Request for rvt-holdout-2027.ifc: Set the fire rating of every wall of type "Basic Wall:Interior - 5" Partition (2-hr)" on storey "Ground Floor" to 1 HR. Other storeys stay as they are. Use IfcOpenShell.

First a look at what the model holds.

```python
import ifcopenshell
import ifcopenshell.util.element

model = ifcopenshell.open("rvt-holdout-2027.ifc")
print(model.schema)
storey = next(s for s in model.by_type("IfcBuildingStorey") if s.Name == "Ground Floor")
walls = [e for e in ifcopenshell.util.element.get_decomposition(storey) if e.is_a("IfcWall")]
seen = {}
for e in walls:
    element_type = ifcopenshell.util.element.get_type(e)
    key = (element_type.Name if element_type != e and element_type else None, ifcopenshell.util.element.get_pset(e, "Pset_WallCommon", "FireRating"))
    seen[key] = seen.get(key, 0) + 1
for (name, value), count in sorted(seen.items(), key=str):
    print(count, "x", name, "|", value)
```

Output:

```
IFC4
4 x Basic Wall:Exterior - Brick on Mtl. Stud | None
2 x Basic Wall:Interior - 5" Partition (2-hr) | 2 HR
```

```python
import ifcopenshell
import ifcopenshell.api.pset
import ifcopenshell.util.element

model = ifcopenshell.open("rvt-holdout-2027.ifc")

storey = next(s for s in model.by_type("IfcBuildingStorey") if s.Name == "Ground Floor")
walls = [e for e in ifcopenshell.util.element.get_decomposition(storey) if e.is_a("IfcWall")]

count = 0
for e in walls:
    element_type = ifcopenshell.util.element.get_type(e)
    if element_type in (None, e) or element_type.Name != 'Basic Wall:Interior - 5" Partition (2-hr)':
        continue
    # add_pset returns the element's existing set when there is one.
    pset = ifcopenshell.api.pset.add_pset(model, product=e, name="Pset_WallCommon")
    ifcopenshell.api.pset.edit_pset(model, pset=pset, properties={"FireRating": "1 HR"})
    count += 1

print(count, "walls updated")

model.write("rvt-holdout-2027-out.ifc")
```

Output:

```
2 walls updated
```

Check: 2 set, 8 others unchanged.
